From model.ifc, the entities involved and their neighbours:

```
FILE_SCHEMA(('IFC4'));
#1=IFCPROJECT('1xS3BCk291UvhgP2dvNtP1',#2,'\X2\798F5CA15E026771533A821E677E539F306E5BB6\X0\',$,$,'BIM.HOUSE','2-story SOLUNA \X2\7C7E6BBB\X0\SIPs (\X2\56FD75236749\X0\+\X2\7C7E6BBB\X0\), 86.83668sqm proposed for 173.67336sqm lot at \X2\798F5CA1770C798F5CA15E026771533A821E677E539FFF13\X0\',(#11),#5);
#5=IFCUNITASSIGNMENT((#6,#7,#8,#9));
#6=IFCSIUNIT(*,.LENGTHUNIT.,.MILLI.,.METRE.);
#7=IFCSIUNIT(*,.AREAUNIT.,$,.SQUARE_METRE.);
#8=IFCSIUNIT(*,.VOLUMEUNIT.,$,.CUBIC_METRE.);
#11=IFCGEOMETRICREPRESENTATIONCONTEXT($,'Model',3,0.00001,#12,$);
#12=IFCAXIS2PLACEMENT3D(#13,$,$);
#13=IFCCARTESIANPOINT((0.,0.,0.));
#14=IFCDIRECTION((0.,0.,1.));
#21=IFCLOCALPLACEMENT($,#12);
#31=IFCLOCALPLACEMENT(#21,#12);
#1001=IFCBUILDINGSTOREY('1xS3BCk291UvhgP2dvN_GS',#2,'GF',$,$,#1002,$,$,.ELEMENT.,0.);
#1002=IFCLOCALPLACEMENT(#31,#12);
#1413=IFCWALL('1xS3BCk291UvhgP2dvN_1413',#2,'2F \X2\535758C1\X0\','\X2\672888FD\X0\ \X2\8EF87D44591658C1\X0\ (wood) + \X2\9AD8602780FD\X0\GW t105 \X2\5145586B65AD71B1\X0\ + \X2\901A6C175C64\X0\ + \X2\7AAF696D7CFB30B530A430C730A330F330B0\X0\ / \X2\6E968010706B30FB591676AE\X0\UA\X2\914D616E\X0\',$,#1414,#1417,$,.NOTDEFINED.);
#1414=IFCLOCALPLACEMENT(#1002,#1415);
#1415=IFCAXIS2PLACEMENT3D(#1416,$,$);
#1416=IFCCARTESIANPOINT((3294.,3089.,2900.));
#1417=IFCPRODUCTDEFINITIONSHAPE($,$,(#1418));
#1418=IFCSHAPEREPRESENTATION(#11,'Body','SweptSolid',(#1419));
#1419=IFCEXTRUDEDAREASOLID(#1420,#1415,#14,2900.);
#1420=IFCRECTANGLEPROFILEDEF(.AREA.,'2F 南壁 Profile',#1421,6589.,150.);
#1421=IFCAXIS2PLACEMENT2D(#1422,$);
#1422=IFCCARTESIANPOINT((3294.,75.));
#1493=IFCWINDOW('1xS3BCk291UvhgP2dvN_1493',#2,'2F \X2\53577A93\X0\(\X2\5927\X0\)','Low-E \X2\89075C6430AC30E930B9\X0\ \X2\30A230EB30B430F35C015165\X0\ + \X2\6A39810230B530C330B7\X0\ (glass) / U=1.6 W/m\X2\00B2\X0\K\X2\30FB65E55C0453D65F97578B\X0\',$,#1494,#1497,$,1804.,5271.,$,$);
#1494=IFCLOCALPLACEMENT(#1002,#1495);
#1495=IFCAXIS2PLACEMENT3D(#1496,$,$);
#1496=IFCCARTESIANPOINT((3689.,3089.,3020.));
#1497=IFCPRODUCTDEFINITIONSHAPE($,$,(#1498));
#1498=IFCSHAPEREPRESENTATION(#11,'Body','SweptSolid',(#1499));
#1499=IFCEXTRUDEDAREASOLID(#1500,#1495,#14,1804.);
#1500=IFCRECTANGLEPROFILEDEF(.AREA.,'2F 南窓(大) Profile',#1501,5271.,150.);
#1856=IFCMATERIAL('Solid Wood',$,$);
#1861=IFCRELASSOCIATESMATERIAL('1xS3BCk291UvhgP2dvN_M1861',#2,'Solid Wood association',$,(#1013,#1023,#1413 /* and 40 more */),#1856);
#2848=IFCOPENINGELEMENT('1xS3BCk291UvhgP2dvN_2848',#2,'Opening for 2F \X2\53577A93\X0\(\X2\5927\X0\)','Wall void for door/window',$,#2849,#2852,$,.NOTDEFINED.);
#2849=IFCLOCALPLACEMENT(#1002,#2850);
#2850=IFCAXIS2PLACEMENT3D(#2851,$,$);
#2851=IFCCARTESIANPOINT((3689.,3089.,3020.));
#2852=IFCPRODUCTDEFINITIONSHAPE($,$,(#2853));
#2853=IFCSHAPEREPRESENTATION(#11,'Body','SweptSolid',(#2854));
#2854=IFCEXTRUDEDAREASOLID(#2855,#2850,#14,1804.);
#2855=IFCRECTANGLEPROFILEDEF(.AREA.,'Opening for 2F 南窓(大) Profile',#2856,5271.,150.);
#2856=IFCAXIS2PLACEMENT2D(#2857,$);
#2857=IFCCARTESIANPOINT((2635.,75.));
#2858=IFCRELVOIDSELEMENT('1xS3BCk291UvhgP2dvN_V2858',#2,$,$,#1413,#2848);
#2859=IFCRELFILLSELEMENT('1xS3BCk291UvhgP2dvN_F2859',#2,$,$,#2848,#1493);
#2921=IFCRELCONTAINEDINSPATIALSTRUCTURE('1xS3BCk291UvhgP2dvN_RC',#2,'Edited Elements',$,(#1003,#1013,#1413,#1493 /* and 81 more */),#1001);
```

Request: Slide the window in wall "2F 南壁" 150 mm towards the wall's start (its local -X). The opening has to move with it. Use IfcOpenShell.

```python
import ifcopenshell
import ifcopenshell.api.geometry
import ifcopenshell.util.placement

model = ifcopenshell.open("model.ifc")

window = model.by_guid("1xS3BCk291UvhgP2dvN_1493")
opening = window.FillsVoids[0].RelatingOpeningElement
wall = opening.VoidsElements[0].RelatingBuildingElement

wall_matrix = ifcopenshell.util.placement.get_local_placement(wall.ObjectPlacement)
shift = wall_matrix[:3, 0] * -150.0
before = ifcopenshell.util.placement.get_local_placement(window.ObjectPlacement)[:3, 3].copy()

# The window is not placed relative to its opening, so move both.
for product in (opening, window):
    matrix = ifcopenshell.util.placement.get_local_placement(product.ObjectPlacement)
    matrix[:3, 3] += shift
    ifcopenshell.api.geometry.edit_object_placement(model, product=product, matrix=matrix, is_si=False)

after = ifcopenshell.util.placement.get_local_placement(window.ObjectPlacement)[:3, 3]
print("window moved by", (after - before).round(3) + 0.0)

model.write("model-out.ifc")
```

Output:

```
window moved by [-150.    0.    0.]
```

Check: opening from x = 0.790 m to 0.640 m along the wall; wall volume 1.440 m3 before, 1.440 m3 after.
